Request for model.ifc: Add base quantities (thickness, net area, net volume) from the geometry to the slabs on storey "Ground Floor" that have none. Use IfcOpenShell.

First a look at what the model holds.

```python
import ifcopenshell
import ifcopenshell.util.element
import ifcopenshell.util.unit

model = ifcopenshell.open("model.ifc")
print(model.schema)
for unit_type in ("LENGTHUNIT", "AREAUNIT", "VOLUMEUNIT"):
    print(unit_type, ifcopenshell.util.unit.calculate_unit_scale(model, unit_type))
storey = next(s for s in model.by_type("IfcBuildingStorey") if s.Name == "Ground Floor")
slabs = [e for e in ifcopenshell.util.element.get_decomposition(storey) if e.is_a("IfcSlab")]
for e in sorted(slabs, key=lambda e: e.id()):
    print(e.id(), e.is_a(), e.Name, list(ifcopenshell.util.element.get_psets(e, qtos_only=True)), sep=" | ")
```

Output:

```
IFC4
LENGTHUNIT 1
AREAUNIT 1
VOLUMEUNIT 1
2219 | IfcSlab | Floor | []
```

```python
import ifcopenshell
import ifcopenshell.api.pset
import ifcopenshell.geom
import ifcopenshell.util.element
import ifcopenshell.util.shape
import ifcopenshell.util.unit

model = ifcopenshell.open("model.ifc")
unit_scale = ifcopenshell.util.unit.calculate_unit_scale(model)
area_scale = ifcopenshell.util.unit.calculate_unit_scale(model, "AREAUNIT")
volume_scale = ifcopenshell.util.unit.calculate_unit_scale(model, "VOLUMEUNIT")
settings = ifcopenshell.geom.settings()

storey = next(s for s in model.by_type("IfcBuildingStorey") if s.Name == "Ground Floor")
slabs = [e for e in ifcopenshell.util.element.get_decomposition(storey) if e.is_a("IfcSlab")]

for e in sorted(slabs, key=lambda e: e.id()):
    if ifcopenshell.util.element.get_psets(e, qtos_only=True, should_inherit=False):
        continue
    # Geometry comes back in metres, in the element's own axes.
    shape = ifcopenshell.geom.create_shape(settings, e)
    values = {
        "Width": ifcopenshell.util.shape.get_z(shape.geometry) / unit_scale,
        "NetArea": ifcopenshell.util.shape.get_footprint_area(shape.geometry) / area_scale,
        "NetVolume": ifcopenshell.util.shape.get_volume(shape.geometry) / volume_scale,
    }
    qto = ifcopenshell.api.pset.add_qto(model, product=e, name="Qto_SlabBaseQuantities")
    ifcopenshell.api.pset.edit_qto(model, qto=qto, properties=values)
    print(e.id(), {k: round(v, 3) for k, v in values.items()})

model.write("model-out.ifc")
```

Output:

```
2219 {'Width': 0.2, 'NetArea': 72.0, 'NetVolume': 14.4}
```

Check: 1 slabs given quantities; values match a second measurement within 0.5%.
